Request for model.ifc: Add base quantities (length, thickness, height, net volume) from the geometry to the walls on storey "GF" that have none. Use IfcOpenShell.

First a look at what the model holds.

```python
import ifcopenshell
import ifcopenshell.util.element
import ifcopenshell.util.unit

model = ifcopenshell.open("model.ifc")
print(model.schema)
for unit_type in ("LENGTHUNIT", "AREAUNIT", "VOLUMEUNIT"):
    print(unit_type, ifcopenshell.util.unit.calculate_unit_scale(model, unit_type))
storey = next(s for s in model.by_type("IfcBuildingStorey") if s.Name == "GF")
walls = [e for e in ifcopenshell.util.element.get_decomposition(storey) if e.is_a("IfcWall")]
for e in sorted(walls, key=lambda e: e.id()):
    print(e.id(), e.is_a(), e.Name, list(ifcopenshell.util.element.get_psets(e, qtos_only=True)), sep=" | ")
```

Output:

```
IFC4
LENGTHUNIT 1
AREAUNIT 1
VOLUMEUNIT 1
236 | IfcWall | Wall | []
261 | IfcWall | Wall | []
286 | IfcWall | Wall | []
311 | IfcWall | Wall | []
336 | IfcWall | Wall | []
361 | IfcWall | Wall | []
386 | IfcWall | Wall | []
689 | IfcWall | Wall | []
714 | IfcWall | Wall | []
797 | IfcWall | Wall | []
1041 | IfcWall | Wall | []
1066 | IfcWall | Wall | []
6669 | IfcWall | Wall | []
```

```python
import ifcopenshell
import ifcopenshell.api.pset
import ifcopenshell.geom
import ifcopenshell.util.element
import ifcopenshell.util.shape
import ifcopenshell.util.unit

model = ifcopenshell.open("model.ifc")
unit_scale = ifcopenshell.util.unit.calculate_unit_scale(model)
volume_scale = ifcopenshell.util.unit.calculate_unit_scale(model, "VOLUMEUNIT")
settings = ifcopenshell.geom.settings()

storey = next(s for s in model.by_type("IfcBuildingStorey") if s.Name == "GF")
walls = [e for e in ifcopenshell.util.element.get_decomposition(storey) if e.is_a("IfcWall")]

for e in sorted(walls, key=lambda e: e.id()):
    if ifcopenshell.util.element.get_psets(e, qtos_only=True, should_inherit=False):
        continue
    # Geometry comes back in metres, in the element's own axes.
    shape = ifcopenshell.geom.create_shape(settings, e)
    values = {
        "Length": ifcopenshell.util.shape.get_x(shape.geometry) / unit_scale,
        "Width": ifcopenshell.util.shape.get_y(shape.geometry) / unit_scale,
        "Height": ifcopenshell.util.shape.get_z(shape.geometry) / unit_scale,
        "NetVolume": ifcopenshell.util.shape.get_volume(shape.geometry) / volume_scale,
    }
    qto = ifcopenshell.api.pset.add_qto(model, product=e, name="Qto_WallBaseQuantities")
    ifcopenshell.api.pset.edit_qto(model, qto=qto, properties=values)
    print(e.id(), {k: round(v, 3) for k, v in values.items()})

model.write("model_rev.ifc")
```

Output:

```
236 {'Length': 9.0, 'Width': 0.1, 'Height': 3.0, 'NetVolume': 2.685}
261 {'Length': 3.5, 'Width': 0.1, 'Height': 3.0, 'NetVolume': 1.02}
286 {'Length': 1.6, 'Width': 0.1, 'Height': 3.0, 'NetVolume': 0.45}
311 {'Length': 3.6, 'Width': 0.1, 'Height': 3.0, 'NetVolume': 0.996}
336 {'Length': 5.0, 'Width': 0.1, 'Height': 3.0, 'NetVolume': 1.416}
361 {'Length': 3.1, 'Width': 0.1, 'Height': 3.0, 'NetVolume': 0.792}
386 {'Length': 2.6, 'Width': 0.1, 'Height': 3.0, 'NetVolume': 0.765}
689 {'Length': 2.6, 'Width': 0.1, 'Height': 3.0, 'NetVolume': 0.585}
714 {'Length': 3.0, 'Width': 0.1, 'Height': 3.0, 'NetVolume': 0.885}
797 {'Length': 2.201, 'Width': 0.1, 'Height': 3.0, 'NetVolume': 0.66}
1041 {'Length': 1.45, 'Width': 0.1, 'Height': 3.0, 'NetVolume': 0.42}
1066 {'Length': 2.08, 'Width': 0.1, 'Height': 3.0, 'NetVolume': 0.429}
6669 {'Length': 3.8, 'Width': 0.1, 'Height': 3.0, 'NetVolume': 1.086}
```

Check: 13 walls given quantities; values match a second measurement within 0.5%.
